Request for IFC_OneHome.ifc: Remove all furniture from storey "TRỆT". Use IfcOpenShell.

First a look at what the model holds.

```python
import ifcopenshell
import ifcopenshell.util.element

model = ifcopenshell.open("IFC_OneHome.ifc")
print(model.schema)
storey = next(s for s in model.by_type("IfcBuildingStorey") if s.Name == "TRỆT")
furniture = [e for e in ifcopenshell.util.element.get_decomposition(storey) if e.is_a("IfcFurnishingElement")]
seen = {}
for e in furniture:
    element_type = ifcopenshell.util.element.get_type(e)
    name = element_type.Name if element_type not in (None, e) else None
    seen[name] = seen.get(name, 0) + 1
for name, count in sorted(seen.items(), key=str):
    print(count, "x", name)
```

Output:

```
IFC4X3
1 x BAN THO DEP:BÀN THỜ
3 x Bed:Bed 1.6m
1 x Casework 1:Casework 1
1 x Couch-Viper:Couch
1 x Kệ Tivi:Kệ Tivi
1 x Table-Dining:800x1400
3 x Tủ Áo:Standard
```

```python
import ifcopenshell
import ifcopenshell.api.root
import ifcopenshell.util.element

model = ifcopenshell.open("IFC_OneHome.ifc")

storey = next(s for s in model.by_type("IfcBuildingStorey") if s.Name == "TRỆT")
furniture = [e for e in ifcopenshell.util.element.get_decomposition(storey) if e.is_a("IfcFurnishingElement")]

for e in furniture:
    ifcopenshell.api.root.remove_product(model, product=e)
print(len(furniture), "removed")

model.write("IFC_OneHome-out.ifc")
```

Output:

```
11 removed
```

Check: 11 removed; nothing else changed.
